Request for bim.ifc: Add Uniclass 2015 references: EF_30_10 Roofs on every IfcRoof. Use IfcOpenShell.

First a look at what the model holds.

```python
import ifcopenshell

model = ifcopenshell.open("bim.ifc")
print(model.schema)
print("classifications:", [c.Name for c in model.by_type("IfcClassification")])
for ifc_class in ("IfcDoor", "IfcRoof", "IfcStair", "IfcWall", "IfcWindow"):
    print(ifc_class, len(model.by_type(ifc_class)))
```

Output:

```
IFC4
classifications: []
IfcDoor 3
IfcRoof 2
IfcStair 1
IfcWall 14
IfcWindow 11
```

```python
import ifcopenshell
import ifcopenshell.api.classification

model = ifcopenshell.open("bim.ifc")

system = ifcopenshell.api.classification.add_classification(model, classification="Uniclass 2015")

codes = {
    "IfcRoof": ("EF_30_10", "Roofs"),
}
for ifc_class, (code, name) in codes.items():
    products = model.by_type(ifc_class)
    ifcopenshell.api.classification.add_reference(
        model, products=products, classification=system, identification=code, name=name
    )
    print(code, len(products))

model.write("bim_updated.ifc")
```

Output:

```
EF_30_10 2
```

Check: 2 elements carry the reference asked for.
